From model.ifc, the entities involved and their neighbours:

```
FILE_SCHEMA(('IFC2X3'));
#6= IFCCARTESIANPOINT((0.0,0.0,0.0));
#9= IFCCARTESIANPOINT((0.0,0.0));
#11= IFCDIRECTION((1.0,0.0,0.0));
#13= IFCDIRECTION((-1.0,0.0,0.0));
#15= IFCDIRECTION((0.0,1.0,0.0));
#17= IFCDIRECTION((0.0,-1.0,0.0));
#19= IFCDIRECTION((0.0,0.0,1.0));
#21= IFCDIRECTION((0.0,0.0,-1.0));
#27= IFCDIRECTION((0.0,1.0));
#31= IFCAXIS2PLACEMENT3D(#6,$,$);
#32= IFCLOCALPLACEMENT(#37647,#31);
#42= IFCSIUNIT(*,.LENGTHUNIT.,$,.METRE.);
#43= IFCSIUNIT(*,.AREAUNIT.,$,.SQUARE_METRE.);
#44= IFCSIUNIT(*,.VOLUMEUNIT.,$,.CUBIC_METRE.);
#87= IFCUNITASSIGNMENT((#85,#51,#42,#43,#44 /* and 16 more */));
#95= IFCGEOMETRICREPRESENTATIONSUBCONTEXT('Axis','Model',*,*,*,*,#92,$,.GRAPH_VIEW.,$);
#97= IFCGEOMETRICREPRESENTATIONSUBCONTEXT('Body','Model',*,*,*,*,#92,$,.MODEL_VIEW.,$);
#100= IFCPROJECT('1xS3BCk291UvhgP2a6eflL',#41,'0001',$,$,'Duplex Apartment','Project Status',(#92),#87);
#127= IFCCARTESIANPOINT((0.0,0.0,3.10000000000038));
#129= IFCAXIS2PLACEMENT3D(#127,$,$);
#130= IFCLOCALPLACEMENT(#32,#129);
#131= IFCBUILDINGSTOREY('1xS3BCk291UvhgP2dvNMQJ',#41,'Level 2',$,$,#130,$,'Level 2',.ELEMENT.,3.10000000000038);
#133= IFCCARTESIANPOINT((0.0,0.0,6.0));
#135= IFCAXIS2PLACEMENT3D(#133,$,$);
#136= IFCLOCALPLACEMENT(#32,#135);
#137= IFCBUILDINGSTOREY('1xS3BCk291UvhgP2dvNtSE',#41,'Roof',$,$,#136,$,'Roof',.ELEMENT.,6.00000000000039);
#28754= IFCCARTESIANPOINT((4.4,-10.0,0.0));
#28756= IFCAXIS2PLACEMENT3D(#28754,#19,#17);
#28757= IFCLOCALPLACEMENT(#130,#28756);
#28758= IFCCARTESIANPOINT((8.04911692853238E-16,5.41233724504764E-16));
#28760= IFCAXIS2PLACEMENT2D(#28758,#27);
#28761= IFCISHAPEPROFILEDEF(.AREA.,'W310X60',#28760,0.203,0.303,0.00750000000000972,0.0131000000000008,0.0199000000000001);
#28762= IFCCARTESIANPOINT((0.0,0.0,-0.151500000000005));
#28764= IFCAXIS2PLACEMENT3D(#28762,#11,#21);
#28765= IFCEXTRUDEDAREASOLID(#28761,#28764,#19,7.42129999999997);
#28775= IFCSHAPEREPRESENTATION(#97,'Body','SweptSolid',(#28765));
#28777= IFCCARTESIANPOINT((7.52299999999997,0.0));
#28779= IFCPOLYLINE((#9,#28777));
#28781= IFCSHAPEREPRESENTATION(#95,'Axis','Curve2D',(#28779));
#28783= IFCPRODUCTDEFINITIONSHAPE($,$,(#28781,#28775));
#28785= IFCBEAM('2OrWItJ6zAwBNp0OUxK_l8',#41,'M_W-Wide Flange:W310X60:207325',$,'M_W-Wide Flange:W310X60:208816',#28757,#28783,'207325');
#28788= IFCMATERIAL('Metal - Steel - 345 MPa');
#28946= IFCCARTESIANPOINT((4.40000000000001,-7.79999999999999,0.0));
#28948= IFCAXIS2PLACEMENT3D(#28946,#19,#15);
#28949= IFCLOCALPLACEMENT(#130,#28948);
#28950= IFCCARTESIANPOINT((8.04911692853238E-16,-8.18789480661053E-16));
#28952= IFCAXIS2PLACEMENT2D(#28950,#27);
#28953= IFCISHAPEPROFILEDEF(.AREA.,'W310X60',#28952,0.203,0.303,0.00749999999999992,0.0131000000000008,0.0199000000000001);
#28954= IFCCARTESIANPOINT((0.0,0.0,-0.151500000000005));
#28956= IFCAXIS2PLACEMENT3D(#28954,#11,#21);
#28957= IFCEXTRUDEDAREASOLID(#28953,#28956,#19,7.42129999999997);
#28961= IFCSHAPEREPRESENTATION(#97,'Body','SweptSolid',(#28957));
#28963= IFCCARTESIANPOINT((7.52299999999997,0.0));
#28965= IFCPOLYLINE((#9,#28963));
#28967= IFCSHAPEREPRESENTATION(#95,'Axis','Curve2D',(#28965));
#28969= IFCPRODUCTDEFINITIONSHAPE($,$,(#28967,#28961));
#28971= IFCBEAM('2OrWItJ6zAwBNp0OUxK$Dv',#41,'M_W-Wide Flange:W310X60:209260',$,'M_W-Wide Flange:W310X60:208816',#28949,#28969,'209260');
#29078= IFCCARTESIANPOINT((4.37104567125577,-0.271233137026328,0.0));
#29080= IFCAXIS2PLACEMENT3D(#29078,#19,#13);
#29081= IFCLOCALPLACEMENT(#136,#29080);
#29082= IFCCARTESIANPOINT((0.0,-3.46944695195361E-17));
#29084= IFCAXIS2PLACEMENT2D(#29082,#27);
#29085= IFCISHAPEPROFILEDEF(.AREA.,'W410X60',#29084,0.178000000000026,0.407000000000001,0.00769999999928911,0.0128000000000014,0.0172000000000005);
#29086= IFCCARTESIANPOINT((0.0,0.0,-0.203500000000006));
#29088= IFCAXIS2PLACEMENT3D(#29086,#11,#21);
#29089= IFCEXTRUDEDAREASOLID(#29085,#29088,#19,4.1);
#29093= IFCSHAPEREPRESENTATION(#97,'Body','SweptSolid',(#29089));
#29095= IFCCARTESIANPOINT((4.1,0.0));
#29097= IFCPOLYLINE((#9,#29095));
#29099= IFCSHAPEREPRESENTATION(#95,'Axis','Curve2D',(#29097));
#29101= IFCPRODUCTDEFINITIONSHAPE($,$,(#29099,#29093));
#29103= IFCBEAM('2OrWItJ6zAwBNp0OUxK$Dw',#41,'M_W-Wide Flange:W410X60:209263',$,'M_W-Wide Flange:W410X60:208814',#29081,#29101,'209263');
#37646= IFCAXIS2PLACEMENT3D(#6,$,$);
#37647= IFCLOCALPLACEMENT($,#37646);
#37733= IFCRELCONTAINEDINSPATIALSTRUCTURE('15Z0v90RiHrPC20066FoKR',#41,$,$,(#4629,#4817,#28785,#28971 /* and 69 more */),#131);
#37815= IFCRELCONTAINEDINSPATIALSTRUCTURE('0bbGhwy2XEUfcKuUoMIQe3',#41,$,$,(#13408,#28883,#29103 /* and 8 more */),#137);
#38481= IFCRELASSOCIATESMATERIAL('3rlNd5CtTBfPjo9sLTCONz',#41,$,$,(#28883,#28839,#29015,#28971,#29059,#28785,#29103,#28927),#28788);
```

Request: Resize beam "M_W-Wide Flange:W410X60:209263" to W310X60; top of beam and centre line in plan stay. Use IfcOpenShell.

```python
import ifcopenshell
import ifcopenshell.util.element
import ifcopenshell.util.representation

model = ifcopenshell.open("model.ifc")

member = model.by_guid("2OrWItJ6zAwBNp0OUxK$Dw")
source = next(p for p in model.by_type("IfcIShapeProfileDef") if p.ProfileName == "W310X60")

body = ifcopenshell.util.representation.get_representation(member, "Model", "Body")
solid = body.Items[0]
old_profile = solid.SweptArea

# Copy the section's sizes but keep this member's own profile position.
profile = ifcopenshell.util.element.copy(model, source)
# Profiles are centred, so shift by half the change in depth to hold the top.
shift = (old_profile.OverallDepth - profile.OverallDepth) / 2
x, y = old_profile.Position.Location.Coordinates
up = (-1.0, 0.0)  # upwards, in the solid's own plane
location = model.createIfcCartesianPoint((x + up[0] * shift, y + up[1] * shift))
profile.Position = model.createIfcAxis2Placement2D(location, old_profile.Position.RefDirection)
solid.SweptArea = profile
if not model.get_total_inverses(old_profile):
    ifcopenshell.util.element.remove_deep2(model, old_profile)
member.Name = member.Name.replace("W410X60", "W310X60")
member.ObjectType = member.ObjectType.replace("W410X60", "W310X60")

print(solid.SweptArea)

model.write("model_updated.ifc")
```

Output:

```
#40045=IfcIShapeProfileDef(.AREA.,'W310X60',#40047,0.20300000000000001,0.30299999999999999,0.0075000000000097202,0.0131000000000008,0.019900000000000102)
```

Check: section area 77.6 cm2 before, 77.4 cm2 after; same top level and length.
